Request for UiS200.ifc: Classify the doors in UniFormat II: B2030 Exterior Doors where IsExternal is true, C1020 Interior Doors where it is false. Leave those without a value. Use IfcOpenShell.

First a look at what the model holds.

```python
import ifcopenshell
import ifcopenshell.util.element

model = ifcopenshell.open("UiS200.ifc")
print(model.schema)
print("classifications:", [c.Name for c in model.by_type("IfcClassification")])
values = [ifcopenshell.util.element.get_pset(e, "Pset_DoorCommon", "IsExternal") for e in model.by_type("IfcDoor")]
for value in (True, False, None):
    print("IsExternal", value, values.count(value))
```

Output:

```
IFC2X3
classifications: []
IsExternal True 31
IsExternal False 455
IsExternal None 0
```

```python
import ifcopenshell
import ifcopenshell.api.classification
import ifcopenshell.util.element

model = ifcopenshell.open("UiS200.ifc")

# IFC2X3 requires Source and Edition and has no link from the project to the system.
system = model.create_entity("IfcClassification", Source="ASTM", Edition="E1557", Name="UniFormat II")

doors = model.by_type("IfcDoor")
external = {e: ifcopenshell.util.element.get_pset(e, "Pset_DoorCommon", "IsExternal") for e in doors}
for flag, code, name in ((True, "B2030", "Exterior Doors"), (False, "C1020", "Interior Doors")):
    products = [e for e in doors if external[e] is flag]
    ifcopenshell.api.classification.add_reference(
        model, products=products, classification=system, identification=code, name=name
    )
    print(code, len(products))

model.write("UiS200_edited.ifc")
```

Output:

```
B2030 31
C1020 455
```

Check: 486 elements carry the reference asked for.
